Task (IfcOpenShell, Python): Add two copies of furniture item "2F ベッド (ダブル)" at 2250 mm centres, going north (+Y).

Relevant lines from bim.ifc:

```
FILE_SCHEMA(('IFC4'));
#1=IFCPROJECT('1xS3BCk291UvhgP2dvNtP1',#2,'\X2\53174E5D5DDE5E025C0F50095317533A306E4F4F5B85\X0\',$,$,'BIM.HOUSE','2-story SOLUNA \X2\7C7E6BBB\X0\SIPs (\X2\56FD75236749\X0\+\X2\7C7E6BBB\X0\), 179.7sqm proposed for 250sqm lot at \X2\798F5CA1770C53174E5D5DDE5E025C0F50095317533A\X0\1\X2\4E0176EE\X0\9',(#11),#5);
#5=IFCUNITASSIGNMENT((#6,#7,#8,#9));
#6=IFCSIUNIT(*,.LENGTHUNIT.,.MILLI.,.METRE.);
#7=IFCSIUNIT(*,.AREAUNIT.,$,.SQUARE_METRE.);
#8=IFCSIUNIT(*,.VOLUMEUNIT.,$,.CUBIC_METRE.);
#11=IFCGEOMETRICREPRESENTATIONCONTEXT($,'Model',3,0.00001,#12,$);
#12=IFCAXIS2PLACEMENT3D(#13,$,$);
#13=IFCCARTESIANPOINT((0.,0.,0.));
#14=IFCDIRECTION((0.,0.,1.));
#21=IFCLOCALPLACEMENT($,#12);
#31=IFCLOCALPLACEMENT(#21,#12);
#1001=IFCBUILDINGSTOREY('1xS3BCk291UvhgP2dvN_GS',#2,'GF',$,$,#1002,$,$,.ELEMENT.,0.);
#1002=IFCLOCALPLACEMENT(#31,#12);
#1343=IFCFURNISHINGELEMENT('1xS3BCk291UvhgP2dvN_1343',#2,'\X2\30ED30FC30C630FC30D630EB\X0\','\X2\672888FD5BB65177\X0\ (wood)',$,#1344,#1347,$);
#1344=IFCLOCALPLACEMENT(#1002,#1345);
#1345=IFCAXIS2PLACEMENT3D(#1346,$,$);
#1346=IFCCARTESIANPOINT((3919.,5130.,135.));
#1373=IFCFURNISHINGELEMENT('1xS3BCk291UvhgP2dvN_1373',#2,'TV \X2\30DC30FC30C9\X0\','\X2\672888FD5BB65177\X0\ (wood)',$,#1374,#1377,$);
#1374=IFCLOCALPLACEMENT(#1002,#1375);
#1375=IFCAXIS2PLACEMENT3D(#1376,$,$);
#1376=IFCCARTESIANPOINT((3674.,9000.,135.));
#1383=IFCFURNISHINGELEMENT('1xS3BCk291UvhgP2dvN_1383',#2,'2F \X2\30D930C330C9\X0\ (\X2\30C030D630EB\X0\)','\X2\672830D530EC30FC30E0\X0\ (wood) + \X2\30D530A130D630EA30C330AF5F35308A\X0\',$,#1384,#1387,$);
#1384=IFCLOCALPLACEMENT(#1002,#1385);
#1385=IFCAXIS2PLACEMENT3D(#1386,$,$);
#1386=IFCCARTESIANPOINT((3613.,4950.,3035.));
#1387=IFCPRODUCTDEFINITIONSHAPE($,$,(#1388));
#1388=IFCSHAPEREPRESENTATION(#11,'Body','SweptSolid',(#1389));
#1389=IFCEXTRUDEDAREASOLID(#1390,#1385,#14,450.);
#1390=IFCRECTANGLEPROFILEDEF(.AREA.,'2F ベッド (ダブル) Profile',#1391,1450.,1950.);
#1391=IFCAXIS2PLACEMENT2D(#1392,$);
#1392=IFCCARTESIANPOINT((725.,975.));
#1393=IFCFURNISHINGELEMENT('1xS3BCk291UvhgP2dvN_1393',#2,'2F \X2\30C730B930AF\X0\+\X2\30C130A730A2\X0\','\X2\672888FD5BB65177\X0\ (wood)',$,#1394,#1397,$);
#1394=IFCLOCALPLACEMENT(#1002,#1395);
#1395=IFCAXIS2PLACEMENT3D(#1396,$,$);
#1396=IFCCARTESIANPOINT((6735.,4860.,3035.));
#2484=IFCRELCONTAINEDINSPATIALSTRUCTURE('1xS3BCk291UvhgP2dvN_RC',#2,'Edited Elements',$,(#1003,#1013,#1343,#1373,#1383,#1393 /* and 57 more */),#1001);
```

```python
import numpy as np
import ifcopenshell
import ifcopenshell.api.geometry
import ifcopenshell.api.root
import ifcopenshell.util.element
import ifcopenshell.util.placement
import ifcopenshell.util.unit

model = ifcopenshell.open("bim.ifc")
unit_scale = ifcopenshell.util.unit.calculate_unit_scale(model)


def reuse_history(source, copy):
    """copy_class also copies each property set's owner history, people and application; keep the originals."""
    for rel in copy.IsDefinedBy:
        if rel.is_a("IfcRelDefinesByProperties") and (history := rel.RelatingPropertyDefinition.OwnerHistory):
            rel.RelatingPropertyDefinition.OwnerHistory = source.OwnerHistory
            ifcopenshell.util.element.remove_deep2(model, history)


source = model.by_guid("1xS3BCk291UvhgP2dvN_1383")
base = ifcopenshell.util.placement.get_local_placement(source.ObjectPlacement)
step = np.array([0.0, 1.0, 0.0]) * 2.25 / unit_scale

for i in range(1, 3):
    copy = ifcopenshell.api.root.copy_class(model, product=source)
    copy.Representation = ifcopenshell.util.element.copy_deep(
        model, source.Representation, exclude=["IfcGeometricRepresentationContext", "IfcRepresentationMap"]
    )
    reuse_history(source, copy)
    matrix = base.copy()
    matrix[:3, 3] += i * step
    print("added at", matrix[:3, 3].round(3) + 0.0)
    ifcopenshell.api.geometry.edit_object_placement(model, product=copy, matrix=matrix, is_si=False)

model.write("bim_rev.ifc")
```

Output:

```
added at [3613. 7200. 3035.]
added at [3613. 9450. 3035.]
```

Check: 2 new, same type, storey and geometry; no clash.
